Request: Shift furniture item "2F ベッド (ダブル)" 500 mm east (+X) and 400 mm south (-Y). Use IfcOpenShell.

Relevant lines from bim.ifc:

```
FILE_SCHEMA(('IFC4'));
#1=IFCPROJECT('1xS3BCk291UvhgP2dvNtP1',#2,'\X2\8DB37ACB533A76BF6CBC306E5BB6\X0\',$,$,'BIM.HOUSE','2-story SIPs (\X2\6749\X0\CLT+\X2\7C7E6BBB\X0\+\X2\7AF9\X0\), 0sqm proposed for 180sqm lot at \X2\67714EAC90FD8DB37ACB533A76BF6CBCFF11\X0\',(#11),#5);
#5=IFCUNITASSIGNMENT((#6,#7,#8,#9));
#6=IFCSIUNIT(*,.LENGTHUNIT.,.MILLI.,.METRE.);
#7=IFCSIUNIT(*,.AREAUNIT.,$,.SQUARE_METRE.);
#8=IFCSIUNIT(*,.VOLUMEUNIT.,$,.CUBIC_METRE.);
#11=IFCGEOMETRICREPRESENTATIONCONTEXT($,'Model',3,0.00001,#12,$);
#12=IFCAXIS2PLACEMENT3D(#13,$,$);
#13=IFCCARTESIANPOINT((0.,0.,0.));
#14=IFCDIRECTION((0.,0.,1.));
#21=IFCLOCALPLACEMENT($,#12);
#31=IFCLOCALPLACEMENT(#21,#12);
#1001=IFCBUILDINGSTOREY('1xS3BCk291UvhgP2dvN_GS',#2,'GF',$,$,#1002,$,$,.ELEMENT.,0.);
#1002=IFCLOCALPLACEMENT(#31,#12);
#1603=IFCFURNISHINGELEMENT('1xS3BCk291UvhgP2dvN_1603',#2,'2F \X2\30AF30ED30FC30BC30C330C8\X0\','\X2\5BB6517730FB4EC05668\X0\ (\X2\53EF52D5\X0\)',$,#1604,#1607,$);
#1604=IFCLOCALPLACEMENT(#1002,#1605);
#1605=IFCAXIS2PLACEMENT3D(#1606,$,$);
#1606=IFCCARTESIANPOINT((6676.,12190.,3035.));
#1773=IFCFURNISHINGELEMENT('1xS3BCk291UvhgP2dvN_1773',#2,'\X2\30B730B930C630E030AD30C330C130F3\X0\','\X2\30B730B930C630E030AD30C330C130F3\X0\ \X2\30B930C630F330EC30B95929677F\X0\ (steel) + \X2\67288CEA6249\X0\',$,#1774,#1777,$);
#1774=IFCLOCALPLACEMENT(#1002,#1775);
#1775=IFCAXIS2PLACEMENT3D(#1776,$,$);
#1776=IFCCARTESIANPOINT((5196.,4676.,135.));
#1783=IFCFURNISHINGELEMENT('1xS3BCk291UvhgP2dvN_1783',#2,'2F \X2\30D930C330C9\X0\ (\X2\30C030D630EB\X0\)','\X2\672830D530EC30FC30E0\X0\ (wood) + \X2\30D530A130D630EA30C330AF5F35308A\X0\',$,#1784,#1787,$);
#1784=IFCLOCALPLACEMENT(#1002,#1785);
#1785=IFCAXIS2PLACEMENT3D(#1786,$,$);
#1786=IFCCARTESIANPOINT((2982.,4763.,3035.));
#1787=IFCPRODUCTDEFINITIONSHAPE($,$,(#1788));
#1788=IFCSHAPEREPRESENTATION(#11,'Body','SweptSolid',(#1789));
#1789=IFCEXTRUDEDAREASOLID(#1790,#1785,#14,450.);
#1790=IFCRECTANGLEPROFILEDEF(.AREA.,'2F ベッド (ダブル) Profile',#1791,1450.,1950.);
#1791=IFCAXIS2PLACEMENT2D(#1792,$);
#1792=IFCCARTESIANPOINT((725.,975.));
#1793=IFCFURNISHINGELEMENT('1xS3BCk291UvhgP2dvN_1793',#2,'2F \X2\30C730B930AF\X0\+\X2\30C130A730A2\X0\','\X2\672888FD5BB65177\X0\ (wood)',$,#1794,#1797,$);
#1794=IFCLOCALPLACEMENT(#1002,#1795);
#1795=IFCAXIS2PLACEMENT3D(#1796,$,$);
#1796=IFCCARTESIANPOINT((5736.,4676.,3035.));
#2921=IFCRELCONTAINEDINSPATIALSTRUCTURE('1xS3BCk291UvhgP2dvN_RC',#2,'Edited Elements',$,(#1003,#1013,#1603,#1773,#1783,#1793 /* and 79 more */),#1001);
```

```python
import ifcopenshell
import ifcopenshell.api.geometry
import ifcopenshell.util.placement
import ifcopenshell.util.unit

model = ifcopenshell.open("bim.ifc")
unit_scale = ifcopenshell.util.unit.calculate_unit_scale(model)

item = model.by_guid("1xS3BCk291UvhgP2dvN_1783")
matrix = ifcopenshell.util.placement.get_local_placement(item.ObjectPlacement)
matrix[0, 3] += 0.5 / unit_scale
matrix[1, 3] -= 0.4 / unit_scale
ifcopenshell.api.geometry.edit_object_placement(model, product=item, matrix=matrix, is_si=False)

print(ifcopenshell.util.placement.get_local_placement(item.ObjectPlacement).round(3) + 0.0)

model.write("bim-out.ifc")
```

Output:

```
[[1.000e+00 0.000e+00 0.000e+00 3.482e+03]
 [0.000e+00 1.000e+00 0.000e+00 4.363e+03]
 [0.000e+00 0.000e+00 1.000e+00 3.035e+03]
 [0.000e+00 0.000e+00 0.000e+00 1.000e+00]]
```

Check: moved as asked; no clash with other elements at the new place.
